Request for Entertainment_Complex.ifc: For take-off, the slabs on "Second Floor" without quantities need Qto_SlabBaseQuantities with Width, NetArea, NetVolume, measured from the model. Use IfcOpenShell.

First a look at what the model holds.

```python
import ifcopenshell
import ifcopenshell.util.element
import ifcopenshell.util.unit

model = ifcopenshell.open("Entertainment_Complex.ifc")
print(model.schema)
for unit_type in ("LENGTHUNIT", "AREAUNIT", "VOLUMEUNIT"):
    print(unit_type, ifcopenshell.util.unit.calculate_unit_scale(model, unit_type))
storey = next(s for s in model.by_type("IfcBuildingStorey") if s.Name == "Second Floor")
slabs = [e for e in ifcopenshell.util.element.get_decomposition(storey) if e.is_a("IfcSlab")]
for e in sorted(slabs, key=lambda e: e.id()):
    print(e.id(), e.is_a(), e.Name, list(ifcopenshell.util.element.get_psets(e, qtos_only=True)), sep=" | ")
```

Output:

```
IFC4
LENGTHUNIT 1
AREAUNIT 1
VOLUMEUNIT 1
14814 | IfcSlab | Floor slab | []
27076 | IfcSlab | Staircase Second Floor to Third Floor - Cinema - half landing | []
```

```python
import ifcopenshell
import ifcopenshell.api.pset
import ifcopenshell.geom
import ifcopenshell.util.element
import ifcopenshell.util.shape
import ifcopenshell.util.unit

model = ifcopenshell.open("Entertainment_Complex.ifc")
unit_scale = ifcopenshell.util.unit.calculate_unit_scale(model)
area_scale = ifcopenshell.util.unit.calculate_unit_scale(model, "AREAUNIT")
volume_scale = ifcopenshell.util.unit.calculate_unit_scale(model, "VOLUMEUNIT")
settings = ifcopenshell.geom.settings()

storey = next(s for s in model.by_type("IfcBuildingStorey") if s.Name == "Second Floor")
slabs = [e for e in ifcopenshell.util.element.get_decomposition(storey) if e.is_a("IfcSlab")]

for e in sorted(slabs, key=lambda e: e.id()):
    if ifcopenshell.util.element.get_psets(e, qtos_only=True, should_inherit=False):
        continue
    # Geometry comes back in metres, in the element's own axes.
    shape = ifcopenshell.geom.create_shape(settings, e)
    values = {
        "Width": ifcopenshell.util.shape.get_z(shape.geometry) / unit_scale,
        "NetArea": ifcopenshell.util.shape.get_footprint_area(shape.geometry) / area_scale,
        "NetVolume": ifcopenshell.util.shape.get_volume(shape.geometry) / volume_scale,
    }
    qto = ifcopenshell.api.pset.add_qto(model, product=e, name="Qto_SlabBaseQuantities")
    ifcopenshell.api.pset.edit_qto(model, qto=qto, properties=values)
    print(e.id(), {k: round(v, 3) for k, v in values.items()})

model.write("Entertainment_Complex_rev.ifc")
```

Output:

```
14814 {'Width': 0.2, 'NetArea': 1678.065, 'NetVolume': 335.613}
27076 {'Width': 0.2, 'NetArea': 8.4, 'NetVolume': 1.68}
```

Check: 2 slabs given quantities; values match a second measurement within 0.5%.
